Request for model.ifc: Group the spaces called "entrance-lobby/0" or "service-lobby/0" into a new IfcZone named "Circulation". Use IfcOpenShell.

First a look at what the model holds.

```python
import ifcopenshell

model = ifcopenshell.open("model.ifc")
print(model.schema)
seen = {}
for space in model.by_type("IfcSpace"):
    seen[space.Name] = seen.get(space.Name, 0) + 1
for name, count in sorted(seen.items(), key=str):
    print(count, "x", name)
print("zones:", [z.Name for z in model.by_type("IfcZone")][:20])
```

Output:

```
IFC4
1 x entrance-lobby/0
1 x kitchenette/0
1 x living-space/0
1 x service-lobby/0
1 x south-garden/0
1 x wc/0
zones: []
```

```python
import ifcopenshell
import ifcopenshell.api.group
import ifcopenshell.api.root

model = ifcopenshell.open("model.ifc")

names = {"entrance-lobby/0", "service-lobby/0"}
spaces = [s for s in model.by_type("IfcSpace") if s.Name in names]

zone = ifcopenshell.api.root.create_entity(model, ifc_class="IfcZone", name="Circulation")
ifcopenshell.api.group.assign_group(model, products=spaces, group=zone)
print(len(spaces), "spaces in", zone.Name)

model.write("model_rev.ifc")
```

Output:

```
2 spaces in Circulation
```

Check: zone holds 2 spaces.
